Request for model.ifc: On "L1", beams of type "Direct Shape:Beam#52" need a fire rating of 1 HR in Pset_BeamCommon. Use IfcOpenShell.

First a look at what the model holds.

```python
import ifcopenshell
import ifcopenshell.util.element

model = ifcopenshell.open("model.ifc")
print(model.schema)
storey = next(s for s in model.by_type("IfcBuildingStorey") if s.Name == "L1")
beams = [e for e in ifcopenshell.util.element.get_decomposition(storey) if e.is_a("IfcBeam")]
seen = {}
for e in beams:
    element_type = ifcopenshell.util.element.get_type(e)
    key = (element_type.Name if element_type != e and element_type else None, ifcopenshell.util.element.get_pset(e, "Pset_BeamCommon", "FireRating"))
    seen[key] = seen.get(key, 0) + 1
for (name, value), count in sorted(seen.items(), key=str):
    print(count, "x", name, "|", value)
```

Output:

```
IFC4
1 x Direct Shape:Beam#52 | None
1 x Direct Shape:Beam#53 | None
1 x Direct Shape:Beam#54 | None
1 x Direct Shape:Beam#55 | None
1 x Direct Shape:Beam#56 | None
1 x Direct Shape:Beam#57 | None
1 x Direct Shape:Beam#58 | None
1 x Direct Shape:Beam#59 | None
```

```python
import ifcopenshell
import ifcopenshell.api.pset
import ifcopenshell.util.element

model = ifcopenshell.open("model.ifc")

storey = next(s for s in model.by_type("IfcBuildingStorey") if s.Name == "L1")
beams = [e for e in ifcopenshell.util.element.get_decomposition(storey) if e.is_a("IfcBeam")]

count = 0
for e in beams:
    element_type = ifcopenshell.util.element.get_type(e)
    if element_type in (None, e) or element_type.Name != "Direct Shape:Beam#52":
        continue
    # add_pset returns the element's existing set when there is one.
    pset = ifcopenshell.api.pset.add_pset(model, product=e, name="Pset_BeamCommon")
    ifcopenshell.api.pset.edit_pset(model, pset=pset, properties={"FireRating": "1 HR"})
    count += 1

print(count, "beams updated")

model.write("model_updated.ifc")
```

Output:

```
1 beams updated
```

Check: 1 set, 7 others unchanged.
